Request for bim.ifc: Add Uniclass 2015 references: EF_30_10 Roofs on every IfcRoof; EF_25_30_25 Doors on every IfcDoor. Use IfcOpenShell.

First a look at what the model holds.

```python
import ifcopenshell

model = ifcopenshell.open("bim.ifc")
print(model.schema)
print("classifications:", [c.Name for c in model.by_type("IfcClassification")])
for ifc_class in ("IfcDoor", "IfcRoof", "IfcStair", "IfcWall", "IfcWindow"):
    print(ifc_class, len(model.by_type(ifc_class)))
```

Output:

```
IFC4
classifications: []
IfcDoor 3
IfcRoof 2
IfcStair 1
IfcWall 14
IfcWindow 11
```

```python
import ifcopenshell
import ifcopenshell.api.classification

model = ifcopenshell.open("bim.ifc")

system = ifcopenshell.api.classification.add_classification(model, classification="Uniclass 2015")

codes = {
    "IfcRoof": ("EF_30_10", "Roofs"),
    "IfcDoor": ("EF_25_30_25", "Doors"),
}
for ifc_class, (code, name) in codes.items():
    products = model.by_type(ifc_class)
    ifcopenshell.api.classification.add_reference(
        model, products=products, classification=system, identification=code, name=name
    )
    print(code, len(products))

model.write("bim_edited.ifc")
```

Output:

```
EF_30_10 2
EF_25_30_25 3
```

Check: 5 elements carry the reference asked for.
